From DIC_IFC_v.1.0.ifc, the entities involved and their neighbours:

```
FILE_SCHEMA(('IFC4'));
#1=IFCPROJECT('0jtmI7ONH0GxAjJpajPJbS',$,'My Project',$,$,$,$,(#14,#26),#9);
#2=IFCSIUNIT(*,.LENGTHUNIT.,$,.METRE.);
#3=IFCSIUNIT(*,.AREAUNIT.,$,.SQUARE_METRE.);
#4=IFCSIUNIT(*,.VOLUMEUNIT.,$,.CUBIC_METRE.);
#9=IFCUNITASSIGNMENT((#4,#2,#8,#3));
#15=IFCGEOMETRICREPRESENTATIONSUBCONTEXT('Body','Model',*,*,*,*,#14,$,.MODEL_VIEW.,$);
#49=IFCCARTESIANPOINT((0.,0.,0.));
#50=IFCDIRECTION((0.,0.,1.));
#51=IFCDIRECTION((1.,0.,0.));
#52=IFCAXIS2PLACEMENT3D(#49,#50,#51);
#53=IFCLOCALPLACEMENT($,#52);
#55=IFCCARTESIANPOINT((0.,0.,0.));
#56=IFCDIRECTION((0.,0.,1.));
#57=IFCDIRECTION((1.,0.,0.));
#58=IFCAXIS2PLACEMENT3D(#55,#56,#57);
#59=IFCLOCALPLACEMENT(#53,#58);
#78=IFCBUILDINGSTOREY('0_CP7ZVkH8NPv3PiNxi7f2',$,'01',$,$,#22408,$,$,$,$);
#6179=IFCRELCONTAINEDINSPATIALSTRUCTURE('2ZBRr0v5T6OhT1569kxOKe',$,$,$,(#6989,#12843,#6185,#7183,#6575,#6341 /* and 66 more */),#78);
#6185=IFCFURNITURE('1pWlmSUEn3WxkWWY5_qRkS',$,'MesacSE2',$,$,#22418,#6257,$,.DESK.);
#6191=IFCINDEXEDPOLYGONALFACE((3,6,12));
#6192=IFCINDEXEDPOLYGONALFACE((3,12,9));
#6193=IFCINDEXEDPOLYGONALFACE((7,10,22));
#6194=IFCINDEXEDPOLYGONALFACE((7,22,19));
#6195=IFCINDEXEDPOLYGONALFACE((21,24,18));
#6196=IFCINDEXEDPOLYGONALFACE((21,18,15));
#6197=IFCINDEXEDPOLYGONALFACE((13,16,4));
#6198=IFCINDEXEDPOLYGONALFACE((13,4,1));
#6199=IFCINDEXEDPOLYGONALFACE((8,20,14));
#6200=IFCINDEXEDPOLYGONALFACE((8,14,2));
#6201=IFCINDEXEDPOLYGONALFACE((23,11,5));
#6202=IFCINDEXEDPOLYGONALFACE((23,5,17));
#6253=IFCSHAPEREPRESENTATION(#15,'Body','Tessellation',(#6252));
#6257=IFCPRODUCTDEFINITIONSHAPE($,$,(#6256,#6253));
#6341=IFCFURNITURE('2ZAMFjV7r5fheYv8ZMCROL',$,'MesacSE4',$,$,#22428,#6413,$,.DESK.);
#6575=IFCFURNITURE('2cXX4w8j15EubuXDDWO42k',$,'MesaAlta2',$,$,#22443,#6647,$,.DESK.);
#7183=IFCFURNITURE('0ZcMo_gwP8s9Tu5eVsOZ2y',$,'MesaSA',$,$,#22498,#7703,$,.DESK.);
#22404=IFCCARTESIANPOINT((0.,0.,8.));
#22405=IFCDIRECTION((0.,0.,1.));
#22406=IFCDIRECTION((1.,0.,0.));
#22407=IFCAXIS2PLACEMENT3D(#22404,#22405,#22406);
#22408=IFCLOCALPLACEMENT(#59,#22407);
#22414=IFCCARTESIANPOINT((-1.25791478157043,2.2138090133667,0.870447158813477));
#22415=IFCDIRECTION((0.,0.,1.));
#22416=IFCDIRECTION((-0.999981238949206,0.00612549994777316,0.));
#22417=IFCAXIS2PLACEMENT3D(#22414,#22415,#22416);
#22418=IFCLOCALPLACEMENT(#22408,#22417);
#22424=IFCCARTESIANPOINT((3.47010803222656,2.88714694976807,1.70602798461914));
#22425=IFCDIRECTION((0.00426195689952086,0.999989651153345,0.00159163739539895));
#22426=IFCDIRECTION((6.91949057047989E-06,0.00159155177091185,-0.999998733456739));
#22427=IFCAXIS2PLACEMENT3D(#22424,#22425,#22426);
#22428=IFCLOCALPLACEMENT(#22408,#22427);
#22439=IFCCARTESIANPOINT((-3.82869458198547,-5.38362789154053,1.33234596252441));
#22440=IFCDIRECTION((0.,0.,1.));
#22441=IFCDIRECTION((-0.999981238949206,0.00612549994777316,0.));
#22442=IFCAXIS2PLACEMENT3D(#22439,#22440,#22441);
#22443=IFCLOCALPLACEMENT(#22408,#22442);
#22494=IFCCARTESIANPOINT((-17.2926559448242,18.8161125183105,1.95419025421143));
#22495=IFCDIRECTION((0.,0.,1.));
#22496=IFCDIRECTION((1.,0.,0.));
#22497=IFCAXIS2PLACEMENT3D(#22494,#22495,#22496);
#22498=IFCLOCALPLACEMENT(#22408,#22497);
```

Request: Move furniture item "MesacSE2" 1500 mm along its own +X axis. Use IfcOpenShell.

```python
import ifcopenshell
import ifcopenshell.api.geometry
import ifcopenshell.util.placement

model = ifcopenshell.open("DIC_IFC_v.1.0.ifc")

item = model.by_guid("1pWlmSUEn3WxkWWY5_qRkS")
matrix = ifcopenshell.util.placement.get_local_placement(item.ObjectPlacement)
matrix[:3, 3] += matrix[:3, 0] * 1.5
ifcopenshell.api.geometry.edit_object_placement(model, product=item, matrix=matrix, is_si=False)

print(ifcopenshell.util.placement.get_local_placement(item.ObjectPlacement).round(3) + 0.0)

model.write("DIC_IFC_v.1.0_v2.ifc")
```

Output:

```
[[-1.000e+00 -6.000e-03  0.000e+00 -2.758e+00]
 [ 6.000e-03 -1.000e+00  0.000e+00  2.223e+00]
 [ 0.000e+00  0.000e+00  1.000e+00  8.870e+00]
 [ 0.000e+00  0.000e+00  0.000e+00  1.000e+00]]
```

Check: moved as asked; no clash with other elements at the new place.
